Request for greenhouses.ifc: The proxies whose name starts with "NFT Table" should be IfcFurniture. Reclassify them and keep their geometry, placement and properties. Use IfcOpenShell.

First a look at what the model holds.

```python
import re

import ifcopenshell

model = ifcopenshell.open("greenhouses.ifc")
print(model.schema)
seen = {}
for e in model.by_type("IfcBuildingElementProxy"):
    name = re.sub(r":\d+(:\d+)?$", "", e.Name or "")  # drop the element id that some exporters append
    seen[name] = seen.get(name, 0) + 1
for name, count in sorted(seen.items()):
    print(count, "x", name)
```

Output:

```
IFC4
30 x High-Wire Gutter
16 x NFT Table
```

```python
import ifcopenshell
import ifcopenshell.api.root

model = ifcopenshell.open("greenhouses.ifc")

proxies = [e.id() for e in model.by_type("IfcBuildingElementProxy") if (e.Name or "").startswith("NFT Table")]
for step_id in proxies:
    proxy = model.by_id(step_id)
    ifcopenshell.api.root.reassign_class(model, product=proxy, ifc_class="IfcFurniture")

print(sum(model.by_id(i).is_a("IfcFurniture") for i in proxies), "reclassified")

model.write("greenhouses_rev.ifc")
```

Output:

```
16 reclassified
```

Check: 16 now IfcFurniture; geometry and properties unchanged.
